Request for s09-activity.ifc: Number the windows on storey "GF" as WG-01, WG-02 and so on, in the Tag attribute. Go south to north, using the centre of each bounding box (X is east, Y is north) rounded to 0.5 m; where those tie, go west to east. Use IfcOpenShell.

First a look at what the model holds.

```python
import ifcopenshell
import ifcopenshell.util.element
import ifcopenshell.util.placement

model = ifcopenshell.open("s09-activity.ifc")
print(model.schema)
storey = next(s for s in model.by_type("IfcBuildingStorey") if s.Name == "GF")
windows = [e for e in ifcopenshell.util.element.get_decomposition(storey) if e.is_a("IfcWindow")]
for e in sorted(windows, key=lambda e: e.id()):
    origin = ifcopenshell.util.placement.get_local_placement(e.ObjectPlacement)[:3, 3]
    print(e.id(), e.Tag, e.Name, origin.round(2) + 0.0, sep=" | ")
```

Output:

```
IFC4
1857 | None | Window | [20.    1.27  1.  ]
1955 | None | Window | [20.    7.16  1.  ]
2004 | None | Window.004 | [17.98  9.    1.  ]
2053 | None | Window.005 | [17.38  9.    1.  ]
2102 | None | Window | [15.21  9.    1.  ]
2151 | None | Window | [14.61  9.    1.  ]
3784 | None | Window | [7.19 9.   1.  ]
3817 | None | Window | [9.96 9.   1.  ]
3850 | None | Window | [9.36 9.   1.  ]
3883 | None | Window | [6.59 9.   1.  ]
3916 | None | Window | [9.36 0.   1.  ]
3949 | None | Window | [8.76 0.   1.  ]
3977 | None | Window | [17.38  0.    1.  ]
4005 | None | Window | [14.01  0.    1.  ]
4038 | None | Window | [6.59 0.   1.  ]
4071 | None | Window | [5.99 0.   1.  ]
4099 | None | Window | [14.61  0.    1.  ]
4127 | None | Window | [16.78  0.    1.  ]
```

```python
import ifcopenshell
import ifcopenshell.geom
import ifcopenshell.util.element
import ifcopenshell.util.shape

model = ifcopenshell.open("s09-activity.ifc")
settings = ifcopenshell.geom.settings()
settings.set("use-world-coords", True)


def centre(element):
    shape = ifcopenshell.geom.create_shape(settings, element)
    return ifcopenshell.util.shape.get_bbox_centroid(shape.geometry)


storey = next(s for s in model.by_type("IfcBuildingStorey") if s.Name == "GF")
windows = [e for e in ifcopenshell.util.element.get_decomposition(storey) if e.is_a("IfcWindow")]

# Insertion points can sit at a corner or the storey origin, so sort by the geometry (in metres).
centres = {e: centre(e) for e in windows}
windows.sort(key=lambda e: (round(centres[e][1] / 0.5), centres[e][0]))

for i, e in enumerate(windows, start=1):
    number = f"WG-{i:02d}"
    e.Tag = number
    print(e.id(), number)

model.write("s09-activity-out.ifc")
```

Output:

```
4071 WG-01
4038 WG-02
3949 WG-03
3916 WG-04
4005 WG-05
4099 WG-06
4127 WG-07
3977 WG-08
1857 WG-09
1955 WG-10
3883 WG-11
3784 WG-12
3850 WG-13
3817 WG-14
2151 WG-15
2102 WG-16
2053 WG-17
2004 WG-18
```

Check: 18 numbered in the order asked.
